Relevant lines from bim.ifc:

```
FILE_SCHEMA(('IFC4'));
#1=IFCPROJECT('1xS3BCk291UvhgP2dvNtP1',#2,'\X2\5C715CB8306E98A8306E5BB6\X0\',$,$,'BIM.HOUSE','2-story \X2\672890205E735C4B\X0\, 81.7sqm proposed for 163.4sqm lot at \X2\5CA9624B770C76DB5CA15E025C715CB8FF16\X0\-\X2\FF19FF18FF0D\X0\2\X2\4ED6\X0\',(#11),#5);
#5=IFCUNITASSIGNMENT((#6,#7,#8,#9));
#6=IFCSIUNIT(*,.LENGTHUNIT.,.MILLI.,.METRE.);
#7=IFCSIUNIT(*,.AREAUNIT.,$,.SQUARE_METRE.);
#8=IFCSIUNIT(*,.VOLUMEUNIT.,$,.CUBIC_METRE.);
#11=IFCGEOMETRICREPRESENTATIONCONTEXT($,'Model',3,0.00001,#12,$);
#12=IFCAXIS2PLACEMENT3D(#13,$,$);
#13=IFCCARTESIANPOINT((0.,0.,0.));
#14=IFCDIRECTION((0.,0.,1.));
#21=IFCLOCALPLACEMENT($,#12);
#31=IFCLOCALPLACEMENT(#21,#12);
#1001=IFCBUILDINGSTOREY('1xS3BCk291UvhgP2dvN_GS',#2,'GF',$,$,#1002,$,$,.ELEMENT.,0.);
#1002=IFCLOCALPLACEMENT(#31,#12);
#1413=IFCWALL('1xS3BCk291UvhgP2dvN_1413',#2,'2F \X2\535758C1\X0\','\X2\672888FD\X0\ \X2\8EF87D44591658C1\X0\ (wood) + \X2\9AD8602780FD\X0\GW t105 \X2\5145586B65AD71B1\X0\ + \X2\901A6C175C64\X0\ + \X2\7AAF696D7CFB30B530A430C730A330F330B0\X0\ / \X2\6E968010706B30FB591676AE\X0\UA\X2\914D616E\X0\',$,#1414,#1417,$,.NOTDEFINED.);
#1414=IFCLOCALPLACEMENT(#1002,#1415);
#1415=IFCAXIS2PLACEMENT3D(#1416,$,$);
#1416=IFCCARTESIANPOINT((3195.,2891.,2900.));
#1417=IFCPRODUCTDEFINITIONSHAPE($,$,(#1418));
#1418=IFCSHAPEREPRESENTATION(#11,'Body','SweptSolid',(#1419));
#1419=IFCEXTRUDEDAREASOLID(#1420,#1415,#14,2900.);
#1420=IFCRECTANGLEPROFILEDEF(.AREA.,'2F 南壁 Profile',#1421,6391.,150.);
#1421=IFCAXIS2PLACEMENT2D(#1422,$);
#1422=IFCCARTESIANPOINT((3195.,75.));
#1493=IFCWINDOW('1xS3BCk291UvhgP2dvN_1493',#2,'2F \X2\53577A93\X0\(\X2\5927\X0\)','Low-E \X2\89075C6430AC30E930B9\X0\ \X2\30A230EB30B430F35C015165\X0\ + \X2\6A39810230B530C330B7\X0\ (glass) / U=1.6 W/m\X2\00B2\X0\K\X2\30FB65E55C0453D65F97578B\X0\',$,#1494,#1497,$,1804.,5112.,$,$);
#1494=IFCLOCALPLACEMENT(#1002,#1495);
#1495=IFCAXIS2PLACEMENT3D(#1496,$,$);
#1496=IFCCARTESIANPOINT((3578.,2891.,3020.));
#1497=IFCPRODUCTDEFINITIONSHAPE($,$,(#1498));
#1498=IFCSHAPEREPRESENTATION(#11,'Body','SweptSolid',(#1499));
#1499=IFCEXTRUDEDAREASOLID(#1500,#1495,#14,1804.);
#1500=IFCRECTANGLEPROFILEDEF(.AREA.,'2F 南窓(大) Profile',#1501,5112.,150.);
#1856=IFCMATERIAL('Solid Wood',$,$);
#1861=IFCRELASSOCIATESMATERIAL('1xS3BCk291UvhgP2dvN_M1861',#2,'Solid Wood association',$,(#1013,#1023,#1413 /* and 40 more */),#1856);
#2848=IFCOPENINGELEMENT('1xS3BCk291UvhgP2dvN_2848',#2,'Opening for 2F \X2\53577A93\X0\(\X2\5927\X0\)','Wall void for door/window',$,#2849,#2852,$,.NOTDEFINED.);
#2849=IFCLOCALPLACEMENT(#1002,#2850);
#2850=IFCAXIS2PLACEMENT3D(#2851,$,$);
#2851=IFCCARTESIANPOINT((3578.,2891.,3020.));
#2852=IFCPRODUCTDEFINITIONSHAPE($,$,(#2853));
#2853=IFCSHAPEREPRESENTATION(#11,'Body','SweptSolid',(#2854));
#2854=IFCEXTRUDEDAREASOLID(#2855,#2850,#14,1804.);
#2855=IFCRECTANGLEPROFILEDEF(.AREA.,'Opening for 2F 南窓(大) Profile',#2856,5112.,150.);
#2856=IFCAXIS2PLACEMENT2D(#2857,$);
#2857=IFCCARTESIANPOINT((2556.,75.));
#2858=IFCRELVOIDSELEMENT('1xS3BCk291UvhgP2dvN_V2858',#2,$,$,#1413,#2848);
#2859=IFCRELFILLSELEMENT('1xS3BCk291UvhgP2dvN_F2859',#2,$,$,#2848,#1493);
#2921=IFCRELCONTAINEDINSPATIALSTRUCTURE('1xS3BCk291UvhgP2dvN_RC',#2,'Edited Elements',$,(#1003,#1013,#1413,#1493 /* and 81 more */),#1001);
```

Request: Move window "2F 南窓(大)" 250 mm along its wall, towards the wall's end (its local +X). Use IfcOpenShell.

```python
import ifcopenshell
import ifcopenshell.api.geometry
import ifcopenshell.util.placement
import ifcopenshell.util.unit

model = ifcopenshell.open("bim.ifc")
unit_scale = ifcopenshell.util.unit.calculate_unit_scale(model)

window = model.by_guid("1xS3BCk291UvhgP2dvN_1493")
opening = window.FillsVoids[0].RelatingOpeningElement
wall = opening.VoidsElements[0].RelatingBuildingElement

wall_matrix = ifcopenshell.util.placement.get_local_placement(wall.ObjectPlacement)
shift = wall_matrix[:3, 0] * 0.25 / unit_scale
before = ifcopenshell.util.placement.get_local_placement(window.ObjectPlacement)[:3, 3].copy()

# The window is not placed relative to its opening, so move both.
for product in (opening, window):
    matrix = ifcopenshell.util.placement.get_local_placement(product.ObjectPlacement)
    matrix[:3, 3] += shift
    ifcopenshell.api.geometry.edit_object_placement(model, product=product, matrix=matrix, is_si=False)

after = ifcopenshell.util.placement.get_local_placement(window.ObjectPlacement)[:3, 3]
print("window moved by", (after - before).round(3) + 0.0)

model.write("bim_rev.ifc")
```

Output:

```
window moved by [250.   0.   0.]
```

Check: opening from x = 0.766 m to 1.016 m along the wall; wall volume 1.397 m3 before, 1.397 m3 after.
